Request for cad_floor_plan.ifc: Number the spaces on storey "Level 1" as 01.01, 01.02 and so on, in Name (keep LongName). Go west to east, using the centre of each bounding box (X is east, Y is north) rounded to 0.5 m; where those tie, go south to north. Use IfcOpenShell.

First a look at what the model holds.

```python
import ifcopenshell
import ifcopenshell.util.element
import ifcopenshell.util.placement

model = ifcopenshell.open("cad_floor_plan.ifc")
print(model.schema)
storey = next(s for s in model.by_type("IfcBuildingStorey") if s.Name == "Level 1")
spaces = [e for e in ifcopenshell.util.element.get_decomposition(storey) if e.is_a("IfcSpace")]
for e in sorted(spaces, key=lambda e: e.id()):
    origin = ifcopenshell.util.placement.get_local_placement(e.ObjectPlacement)[:3, 3]
    print(e.id(), e.Name, e.LongName, origin.round(2) + 0.0, sep=" | ")
```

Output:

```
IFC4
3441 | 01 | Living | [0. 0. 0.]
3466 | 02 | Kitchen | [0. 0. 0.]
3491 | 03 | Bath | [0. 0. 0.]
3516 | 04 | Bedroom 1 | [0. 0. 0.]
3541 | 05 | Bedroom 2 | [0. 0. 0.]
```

```python
import ifcopenshell
import ifcopenshell.geom
import ifcopenshell.util.element
import ifcopenshell.util.shape

model = ifcopenshell.open("cad_floor_plan.ifc")
settings = ifcopenshell.geom.settings()
settings.set("use-world-coords", True)


def centre(element):
    shape = ifcopenshell.geom.create_shape(settings, element)
    return ifcopenshell.util.shape.get_bbox_centroid(shape.geometry)


storey = next(s for s in model.by_type("IfcBuildingStorey") if s.Name == "Level 1")
spaces = [e for e in ifcopenshell.util.element.get_decomposition(storey) if e.is_a("IfcSpace")]

# Insertion points can sit at a corner or the storey origin, so sort by the geometry (in metres).
centres = {e: centre(e) for e in spaces}
spaces.sort(key=lambda e: (round(centres[e][0] / 0.5), centres[e][1]))

for i, e in enumerate(spaces, start=1):
    number = f"01.{i:02d}"
    e.Name = number
    print(e.id(), number)

model.write("cad_floor_plan_v2.ifc")
```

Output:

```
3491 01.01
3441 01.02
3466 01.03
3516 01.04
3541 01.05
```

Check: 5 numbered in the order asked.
